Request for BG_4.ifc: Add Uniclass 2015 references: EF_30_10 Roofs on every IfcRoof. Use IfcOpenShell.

First a look at what the model holds.

```python
import ifcopenshell

model = ifcopenshell.open("BG_4.ifc")
print(model.schema)
print("classifications:", [c.Name for c in model.by_type("IfcClassification")])
for ifc_class in ("IfcDoor", "IfcRoof", "IfcStair", "IfcWall", "IfcWindow"):
    print(ifc_class, len(model.by_type(ifc_class)))
```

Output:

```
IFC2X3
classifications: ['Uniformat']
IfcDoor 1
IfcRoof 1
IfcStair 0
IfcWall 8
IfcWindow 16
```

```python
import ifcopenshell
import ifcopenshell.api.classification

model = ifcopenshell.open("BG_4.ifc")

# IFC2X3 requires Source and Edition and has no link from the project to the system.
system = model.create_entity("IfcClassification", Source="NBS", Edition="2015", Name="Uniclass 2015")

codes = {
    "IfcRoof": ("EF_30_10", "Roofs"),
}
for ifc_class, (code, name) in codes.items():
    products = model.by_type(ifc_class)
    ifcopenshell.api.classification.add_reference(
        model, products=products, classification=system, identification=code, name=name
    )
    print(code, len(products))

model.write("BG_4_v2.ifc")
```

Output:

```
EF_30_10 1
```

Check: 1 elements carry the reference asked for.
